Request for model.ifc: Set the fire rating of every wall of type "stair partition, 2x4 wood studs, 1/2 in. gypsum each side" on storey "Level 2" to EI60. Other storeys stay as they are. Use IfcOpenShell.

First a look at what the model holds.

```python
import ifcopenshell
import ifcopenshell.util.element

model = ifcopenshell.open("model.ifc")
print(model.schema)
storey = next(s for s in model.by_type("IfcBuildingStorey") if s.Name == "Level 2")
walls = [e for e in ifcopenshell.util.element.get_decomposition(storey) if e.is_a("IfcWall")]
seen = {}
for e in walls:
    element_type = ifcopenshell.util.element.get_type(e)
    key = (element_type.Name if element_type != e and element_type else None, ifcopenshell.util.element.get_pset(e, "Pset_WallCommon", "FireRating"))
    seen[key] = seen.get(key, 0) + 1
for (name, value), count in sorted(seen.items(), key=str):
    print(count, "x", name, "|", value)
```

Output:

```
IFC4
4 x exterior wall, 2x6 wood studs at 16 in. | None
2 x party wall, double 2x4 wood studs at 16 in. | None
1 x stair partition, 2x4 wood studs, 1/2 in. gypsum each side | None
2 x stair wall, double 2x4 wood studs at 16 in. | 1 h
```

```python
import ifcopenshell
import ifcopenshell.api.pset
import ifcopenshell.util.element

model = ifcopenshell.open("model.ifc")

storey = next(s for s in model.by_type("IfcBuildingStorey") if s.Name == "Level 2")
walls = [e for e in ifcopenshell.util.element.get_decomposition(storey) if e.is_a("IfcWall")]

count = 0
for e in walls:
    element_type = ifcopenshell.util.element.get_type(e)
    if element_type in (None, e) or element_type.Name != "stair partition, 2x4 wood studs, 1/2 in. gypsum each side":
        continue
    # add_pset returns the element's existing set when there is one.
    pset = ifcopenshell.api.pset.add_pset(model, product=e, name="Pset_WallCommon")
    ifcopenshell.api.pset.edit_pset(model, pset=pset, properties={"FireRating": "EI60"})
    count += 1

print(count, "walls updated")

model.write("model_updated.ifc")
```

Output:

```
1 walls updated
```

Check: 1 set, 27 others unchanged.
